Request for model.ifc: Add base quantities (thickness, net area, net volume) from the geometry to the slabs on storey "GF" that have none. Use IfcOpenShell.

First a look at what the model holds.

```python
import ifcopenshell
import ifcopenshell.util.element
import ifcopenshell.util.unit

model = ifcopenshell.open("model.ifc")
print(model.schema)
for unit_type in ("LENGTHUNIT", "AREAUNIT", "VOLUMEUNIT"):
    print(unit_type, ifcopenshell.util.unit.calculate_unit_scale(model, unit_type))
storey = next(s for s in model.by_type("IfcBuildingStorey") if s.Name == "GF")
slabs = [e for e in ifcopenshell.util.element.get_decomposition(storey) if e.is_a("IfcSlab")]
for e in sorted(slabs, key=lambda e: e.id()):
    print(e.id(), e.is_a(), e.Name, list(ifcopenshell.util.element.get_psets(e, qtos_only=True)), sep=" | ")
```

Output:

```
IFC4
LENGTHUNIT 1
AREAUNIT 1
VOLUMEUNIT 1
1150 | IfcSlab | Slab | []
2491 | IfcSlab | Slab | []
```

```python
import ifcopenshell
import ifcopenshell.api.pset
import ifcopenshell.geom
import ifcopenshell.util.element
import ifcopenshell.util.shape
import ifcopenshell.util.unit

model = ifcopenshell.open("model.ifc")
unit_scale = ifcopenshell.util.unit.calculate_unit_scale(model)
area_scale = ifcopenshell.util.unit.calculate_unit_scale(model, "AREAUNIT")
volume_scale = ifcopenshell.util.unit.calculate_unit_scale(model, "VOLUMEUNIT")
settings = ifcopenshell.geom.settings()

storey = next(s for s in model.by_type("IfcBuildingStorey") if s.Name == "GF")
slabs = [e for e in ifcopenshell.util.element.get_decomposition(storey) if e.is_a("IfcSlab")]

for e in sorted(slabs, key=lambda e: e.id()):
    if ifcopenshell.util.element.get_psets(e, qtos_only=True, should_inherit=False):
        continue
    # Geometry comes back in metres, in the element's own axes.
    shape = ifcopenshell.geom.create_shape(settings, e)
    values = {
        "Width": ifcopenshell.util.shape.get_z(shape.geometry) / unit_scale,
        "NetArea": ifcopenshell.util.shape.get_footprint_area(shape.geometry) / area_scale,
        "NetVolume": ifcopenshell.util.shape.get_volume(shape.geometry) / volume_scale,
    }
    qto = ifcopenshell.api.pset.add_qto(model, product=e, name="Qto_SlabBaseQuantities")
    ifcopenshell.api.pset.edit_qto(model, qto=qto, properties=values)
    print(e.id(), {k: round(v, 3) for k, v in values.items()})

model.write("model_updated.ifc")
```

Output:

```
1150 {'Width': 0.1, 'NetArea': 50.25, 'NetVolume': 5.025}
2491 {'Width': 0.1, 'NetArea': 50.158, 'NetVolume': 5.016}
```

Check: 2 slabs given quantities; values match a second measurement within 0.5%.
